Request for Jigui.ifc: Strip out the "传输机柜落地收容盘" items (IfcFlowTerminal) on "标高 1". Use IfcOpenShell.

First a look at what the model holds.

```python
import ifcopenshell
import ifcopenshell.util.element

model = ifcopenshell.open("Jigui.ifc")
print(model.schema)
storey = next(s for s in model.by_type("IfcBuildingStorey") if s.Name == "标高 1")
terminals = [e for e in ifcopenshell.util.element.get_decomposition(storey) if e.is_a("IfcFlowTerminal")]
seen = {}
for e in terminals:
    element_type = ifcopenshell.util.element.get_type(e)
    name = element_type.Name if element_type not in (None, e) else None
    seen[name] = seen.get(name, 0) + 1
for name, count in sorted(seen.items(), key=str):
    print(count, "x", name)
```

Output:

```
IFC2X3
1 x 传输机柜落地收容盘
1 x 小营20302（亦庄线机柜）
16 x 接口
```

```python
import ifcopenshell
import ifcopenshell.api.root
import ifcopenshell.util.element

model = ifcopenshell.open("Jigui.ifc")

storey = next(s for s in model.by_type("IfcBuildingStorey") if s.Name == "标高 1")
terminals = [e for e in ifcopenshell.util.element.get_decomposition(storey) if e.is_a("IfcFlowTerminal")]
targets = [e for e in terminals if (t := ifcopenshell.util.element.get_type(e)) not in (None, e) and t.Name == "传输机柜落地收容盘"]

for e in targets:
    ifcopenshell.api.root.remove_product(model, product=e)
print(len(targets), "removed")

model.write("Jigui-out.ifc")
```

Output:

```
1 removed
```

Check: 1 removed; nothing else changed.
